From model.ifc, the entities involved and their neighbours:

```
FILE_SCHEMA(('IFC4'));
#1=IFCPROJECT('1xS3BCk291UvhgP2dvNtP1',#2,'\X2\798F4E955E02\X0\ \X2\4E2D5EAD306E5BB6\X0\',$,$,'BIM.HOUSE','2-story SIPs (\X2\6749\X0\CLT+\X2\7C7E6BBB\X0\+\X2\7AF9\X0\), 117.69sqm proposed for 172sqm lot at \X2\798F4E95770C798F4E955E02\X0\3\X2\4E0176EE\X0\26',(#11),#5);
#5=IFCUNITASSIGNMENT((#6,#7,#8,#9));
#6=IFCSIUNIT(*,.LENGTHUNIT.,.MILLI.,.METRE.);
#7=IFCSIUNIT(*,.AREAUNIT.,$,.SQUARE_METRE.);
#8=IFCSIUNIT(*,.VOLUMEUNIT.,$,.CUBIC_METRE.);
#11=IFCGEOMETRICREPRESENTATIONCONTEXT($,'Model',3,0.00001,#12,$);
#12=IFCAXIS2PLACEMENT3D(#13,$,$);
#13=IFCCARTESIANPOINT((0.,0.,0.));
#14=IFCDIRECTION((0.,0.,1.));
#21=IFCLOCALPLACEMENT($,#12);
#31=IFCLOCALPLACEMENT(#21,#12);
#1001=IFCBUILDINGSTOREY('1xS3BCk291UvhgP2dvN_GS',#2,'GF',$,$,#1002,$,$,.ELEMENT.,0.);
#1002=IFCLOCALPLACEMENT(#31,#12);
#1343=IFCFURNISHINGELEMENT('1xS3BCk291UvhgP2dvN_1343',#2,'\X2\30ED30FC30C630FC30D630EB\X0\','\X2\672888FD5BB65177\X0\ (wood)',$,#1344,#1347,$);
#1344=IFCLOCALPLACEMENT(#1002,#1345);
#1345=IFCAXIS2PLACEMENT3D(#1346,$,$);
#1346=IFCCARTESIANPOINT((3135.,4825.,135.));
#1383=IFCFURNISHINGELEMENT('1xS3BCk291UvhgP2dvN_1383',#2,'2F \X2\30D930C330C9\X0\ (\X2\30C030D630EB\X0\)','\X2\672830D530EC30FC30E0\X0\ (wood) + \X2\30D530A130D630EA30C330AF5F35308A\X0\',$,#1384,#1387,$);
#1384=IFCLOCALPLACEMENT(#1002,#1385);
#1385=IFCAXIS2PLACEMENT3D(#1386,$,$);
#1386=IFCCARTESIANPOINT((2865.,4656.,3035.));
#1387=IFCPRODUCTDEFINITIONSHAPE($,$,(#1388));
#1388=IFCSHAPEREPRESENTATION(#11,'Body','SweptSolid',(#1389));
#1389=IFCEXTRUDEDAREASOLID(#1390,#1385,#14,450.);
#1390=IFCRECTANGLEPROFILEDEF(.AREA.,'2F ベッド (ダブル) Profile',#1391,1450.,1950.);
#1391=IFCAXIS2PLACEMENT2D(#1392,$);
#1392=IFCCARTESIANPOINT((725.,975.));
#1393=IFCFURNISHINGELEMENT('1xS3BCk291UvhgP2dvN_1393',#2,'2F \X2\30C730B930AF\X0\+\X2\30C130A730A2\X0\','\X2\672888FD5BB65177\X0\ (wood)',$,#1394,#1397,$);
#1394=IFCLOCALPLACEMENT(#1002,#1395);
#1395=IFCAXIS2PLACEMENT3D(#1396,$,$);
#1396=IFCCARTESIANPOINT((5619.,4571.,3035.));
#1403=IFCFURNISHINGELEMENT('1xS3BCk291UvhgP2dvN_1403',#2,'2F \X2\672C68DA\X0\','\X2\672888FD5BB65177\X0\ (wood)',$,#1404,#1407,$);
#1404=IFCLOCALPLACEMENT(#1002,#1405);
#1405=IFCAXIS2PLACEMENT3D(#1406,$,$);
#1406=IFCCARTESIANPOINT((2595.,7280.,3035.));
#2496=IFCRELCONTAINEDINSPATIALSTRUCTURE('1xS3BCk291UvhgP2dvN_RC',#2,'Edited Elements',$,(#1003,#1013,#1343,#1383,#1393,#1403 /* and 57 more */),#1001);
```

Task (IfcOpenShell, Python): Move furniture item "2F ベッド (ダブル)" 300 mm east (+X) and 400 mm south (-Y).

```python
import ifcopenshell
import ifcopenshell.api.geometry
import ifcopenshell.util.placement
import ifcopenshell.util.unit

model = ifcopenshell.open("model.ifc")
unit_scale = ifcopenshell.util.unit.calculate_unit_scale(model)

item = model.by_guid("1xS3BCk291UvhgP2dvN_1383")
matrix = ifcopenshell.util.placement.get_local_placement(item.ObjectPlacement)
matrix[0, 3] += 0.3 / unit_scale
matrix[1, 3] -= 0.4 / unit_scale
ifcopenshell.api.geometry.edit_object_placement(model, product=item, matrix=matrix, is_si=False)

print(ifcopenshell.util.placement.get_local_placement(item.ObjectPlacement).round(3) + 0.0)

model.write("model_updated.ifc")
```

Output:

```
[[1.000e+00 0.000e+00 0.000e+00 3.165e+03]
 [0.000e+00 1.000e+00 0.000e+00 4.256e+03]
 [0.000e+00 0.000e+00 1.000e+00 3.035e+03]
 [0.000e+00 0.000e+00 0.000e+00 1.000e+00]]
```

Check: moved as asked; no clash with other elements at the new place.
